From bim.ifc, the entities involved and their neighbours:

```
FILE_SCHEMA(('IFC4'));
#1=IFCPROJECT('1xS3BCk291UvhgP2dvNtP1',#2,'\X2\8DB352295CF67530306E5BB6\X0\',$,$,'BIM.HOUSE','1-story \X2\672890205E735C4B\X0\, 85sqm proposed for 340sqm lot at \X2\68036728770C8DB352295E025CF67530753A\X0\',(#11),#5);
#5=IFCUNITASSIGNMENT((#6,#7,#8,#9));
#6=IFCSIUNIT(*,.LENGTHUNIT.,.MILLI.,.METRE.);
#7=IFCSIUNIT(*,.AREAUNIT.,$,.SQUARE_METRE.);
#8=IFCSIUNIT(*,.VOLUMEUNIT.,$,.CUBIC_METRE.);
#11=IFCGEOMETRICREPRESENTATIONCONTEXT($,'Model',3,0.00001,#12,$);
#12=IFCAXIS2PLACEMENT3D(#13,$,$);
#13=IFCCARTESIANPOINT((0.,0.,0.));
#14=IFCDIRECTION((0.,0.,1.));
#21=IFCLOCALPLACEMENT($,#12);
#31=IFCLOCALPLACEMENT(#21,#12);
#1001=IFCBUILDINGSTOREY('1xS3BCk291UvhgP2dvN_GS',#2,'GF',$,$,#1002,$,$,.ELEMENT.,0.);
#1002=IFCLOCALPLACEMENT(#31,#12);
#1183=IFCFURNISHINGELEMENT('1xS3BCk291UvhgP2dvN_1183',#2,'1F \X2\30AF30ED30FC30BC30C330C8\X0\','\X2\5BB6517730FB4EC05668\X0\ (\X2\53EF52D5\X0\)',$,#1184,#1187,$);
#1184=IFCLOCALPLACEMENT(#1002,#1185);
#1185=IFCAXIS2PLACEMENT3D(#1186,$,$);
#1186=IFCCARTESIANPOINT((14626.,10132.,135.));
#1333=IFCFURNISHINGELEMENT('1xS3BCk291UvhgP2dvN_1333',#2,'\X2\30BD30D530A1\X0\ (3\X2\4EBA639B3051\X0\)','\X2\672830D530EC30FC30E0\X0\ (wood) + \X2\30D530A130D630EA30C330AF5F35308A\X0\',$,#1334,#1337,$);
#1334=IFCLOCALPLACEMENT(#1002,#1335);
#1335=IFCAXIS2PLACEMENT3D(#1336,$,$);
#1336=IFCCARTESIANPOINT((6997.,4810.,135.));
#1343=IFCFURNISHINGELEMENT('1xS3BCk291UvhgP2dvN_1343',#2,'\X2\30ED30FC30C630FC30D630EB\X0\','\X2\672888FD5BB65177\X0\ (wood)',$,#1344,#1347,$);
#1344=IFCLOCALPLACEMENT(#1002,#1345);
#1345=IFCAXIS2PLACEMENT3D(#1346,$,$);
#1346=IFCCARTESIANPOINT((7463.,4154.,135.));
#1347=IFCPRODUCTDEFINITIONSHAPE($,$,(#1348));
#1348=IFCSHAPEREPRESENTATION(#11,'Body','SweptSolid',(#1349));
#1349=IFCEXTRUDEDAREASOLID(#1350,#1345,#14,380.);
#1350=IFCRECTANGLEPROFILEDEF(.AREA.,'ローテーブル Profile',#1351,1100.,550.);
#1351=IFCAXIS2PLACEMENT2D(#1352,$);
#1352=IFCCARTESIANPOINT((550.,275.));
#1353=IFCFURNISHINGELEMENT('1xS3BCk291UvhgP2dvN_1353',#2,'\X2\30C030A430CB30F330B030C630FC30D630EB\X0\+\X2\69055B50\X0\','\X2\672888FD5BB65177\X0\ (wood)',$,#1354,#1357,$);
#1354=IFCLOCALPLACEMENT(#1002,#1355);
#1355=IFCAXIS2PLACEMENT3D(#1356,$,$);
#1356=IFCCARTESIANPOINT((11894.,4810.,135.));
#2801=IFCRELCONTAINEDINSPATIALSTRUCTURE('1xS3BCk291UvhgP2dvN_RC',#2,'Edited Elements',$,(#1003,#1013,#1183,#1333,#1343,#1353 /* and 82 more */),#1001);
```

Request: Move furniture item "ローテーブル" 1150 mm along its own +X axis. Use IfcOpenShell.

```python
import ifcopenshell
import ifcopenshell.api.geometry
import ifcopenshell.util.placement

model = ifcopenshell.open("bim.ifc")

item = model.by_guid("1xS3BCk291UvhgP2dvN_1343")
matrix = ifcopenshell.util.placement.get_local_placement(item.ObjectPlacement)
matrix[:3, 3] += matrix[:3, 0] * 1150.0
ifcopenshell.api.geometry.edit_object_placement(model, product=item, matrix=matrix, is_si=False)

print(ifcopenshell.util.placement.get_local_placement(item.ObjectPlacement).round(3) + 0.0)

model.write("bim_v2.ifc")
```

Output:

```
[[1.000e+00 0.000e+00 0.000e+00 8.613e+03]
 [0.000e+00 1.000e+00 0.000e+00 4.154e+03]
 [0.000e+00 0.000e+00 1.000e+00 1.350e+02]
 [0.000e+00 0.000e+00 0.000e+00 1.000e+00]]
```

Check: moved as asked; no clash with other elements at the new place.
